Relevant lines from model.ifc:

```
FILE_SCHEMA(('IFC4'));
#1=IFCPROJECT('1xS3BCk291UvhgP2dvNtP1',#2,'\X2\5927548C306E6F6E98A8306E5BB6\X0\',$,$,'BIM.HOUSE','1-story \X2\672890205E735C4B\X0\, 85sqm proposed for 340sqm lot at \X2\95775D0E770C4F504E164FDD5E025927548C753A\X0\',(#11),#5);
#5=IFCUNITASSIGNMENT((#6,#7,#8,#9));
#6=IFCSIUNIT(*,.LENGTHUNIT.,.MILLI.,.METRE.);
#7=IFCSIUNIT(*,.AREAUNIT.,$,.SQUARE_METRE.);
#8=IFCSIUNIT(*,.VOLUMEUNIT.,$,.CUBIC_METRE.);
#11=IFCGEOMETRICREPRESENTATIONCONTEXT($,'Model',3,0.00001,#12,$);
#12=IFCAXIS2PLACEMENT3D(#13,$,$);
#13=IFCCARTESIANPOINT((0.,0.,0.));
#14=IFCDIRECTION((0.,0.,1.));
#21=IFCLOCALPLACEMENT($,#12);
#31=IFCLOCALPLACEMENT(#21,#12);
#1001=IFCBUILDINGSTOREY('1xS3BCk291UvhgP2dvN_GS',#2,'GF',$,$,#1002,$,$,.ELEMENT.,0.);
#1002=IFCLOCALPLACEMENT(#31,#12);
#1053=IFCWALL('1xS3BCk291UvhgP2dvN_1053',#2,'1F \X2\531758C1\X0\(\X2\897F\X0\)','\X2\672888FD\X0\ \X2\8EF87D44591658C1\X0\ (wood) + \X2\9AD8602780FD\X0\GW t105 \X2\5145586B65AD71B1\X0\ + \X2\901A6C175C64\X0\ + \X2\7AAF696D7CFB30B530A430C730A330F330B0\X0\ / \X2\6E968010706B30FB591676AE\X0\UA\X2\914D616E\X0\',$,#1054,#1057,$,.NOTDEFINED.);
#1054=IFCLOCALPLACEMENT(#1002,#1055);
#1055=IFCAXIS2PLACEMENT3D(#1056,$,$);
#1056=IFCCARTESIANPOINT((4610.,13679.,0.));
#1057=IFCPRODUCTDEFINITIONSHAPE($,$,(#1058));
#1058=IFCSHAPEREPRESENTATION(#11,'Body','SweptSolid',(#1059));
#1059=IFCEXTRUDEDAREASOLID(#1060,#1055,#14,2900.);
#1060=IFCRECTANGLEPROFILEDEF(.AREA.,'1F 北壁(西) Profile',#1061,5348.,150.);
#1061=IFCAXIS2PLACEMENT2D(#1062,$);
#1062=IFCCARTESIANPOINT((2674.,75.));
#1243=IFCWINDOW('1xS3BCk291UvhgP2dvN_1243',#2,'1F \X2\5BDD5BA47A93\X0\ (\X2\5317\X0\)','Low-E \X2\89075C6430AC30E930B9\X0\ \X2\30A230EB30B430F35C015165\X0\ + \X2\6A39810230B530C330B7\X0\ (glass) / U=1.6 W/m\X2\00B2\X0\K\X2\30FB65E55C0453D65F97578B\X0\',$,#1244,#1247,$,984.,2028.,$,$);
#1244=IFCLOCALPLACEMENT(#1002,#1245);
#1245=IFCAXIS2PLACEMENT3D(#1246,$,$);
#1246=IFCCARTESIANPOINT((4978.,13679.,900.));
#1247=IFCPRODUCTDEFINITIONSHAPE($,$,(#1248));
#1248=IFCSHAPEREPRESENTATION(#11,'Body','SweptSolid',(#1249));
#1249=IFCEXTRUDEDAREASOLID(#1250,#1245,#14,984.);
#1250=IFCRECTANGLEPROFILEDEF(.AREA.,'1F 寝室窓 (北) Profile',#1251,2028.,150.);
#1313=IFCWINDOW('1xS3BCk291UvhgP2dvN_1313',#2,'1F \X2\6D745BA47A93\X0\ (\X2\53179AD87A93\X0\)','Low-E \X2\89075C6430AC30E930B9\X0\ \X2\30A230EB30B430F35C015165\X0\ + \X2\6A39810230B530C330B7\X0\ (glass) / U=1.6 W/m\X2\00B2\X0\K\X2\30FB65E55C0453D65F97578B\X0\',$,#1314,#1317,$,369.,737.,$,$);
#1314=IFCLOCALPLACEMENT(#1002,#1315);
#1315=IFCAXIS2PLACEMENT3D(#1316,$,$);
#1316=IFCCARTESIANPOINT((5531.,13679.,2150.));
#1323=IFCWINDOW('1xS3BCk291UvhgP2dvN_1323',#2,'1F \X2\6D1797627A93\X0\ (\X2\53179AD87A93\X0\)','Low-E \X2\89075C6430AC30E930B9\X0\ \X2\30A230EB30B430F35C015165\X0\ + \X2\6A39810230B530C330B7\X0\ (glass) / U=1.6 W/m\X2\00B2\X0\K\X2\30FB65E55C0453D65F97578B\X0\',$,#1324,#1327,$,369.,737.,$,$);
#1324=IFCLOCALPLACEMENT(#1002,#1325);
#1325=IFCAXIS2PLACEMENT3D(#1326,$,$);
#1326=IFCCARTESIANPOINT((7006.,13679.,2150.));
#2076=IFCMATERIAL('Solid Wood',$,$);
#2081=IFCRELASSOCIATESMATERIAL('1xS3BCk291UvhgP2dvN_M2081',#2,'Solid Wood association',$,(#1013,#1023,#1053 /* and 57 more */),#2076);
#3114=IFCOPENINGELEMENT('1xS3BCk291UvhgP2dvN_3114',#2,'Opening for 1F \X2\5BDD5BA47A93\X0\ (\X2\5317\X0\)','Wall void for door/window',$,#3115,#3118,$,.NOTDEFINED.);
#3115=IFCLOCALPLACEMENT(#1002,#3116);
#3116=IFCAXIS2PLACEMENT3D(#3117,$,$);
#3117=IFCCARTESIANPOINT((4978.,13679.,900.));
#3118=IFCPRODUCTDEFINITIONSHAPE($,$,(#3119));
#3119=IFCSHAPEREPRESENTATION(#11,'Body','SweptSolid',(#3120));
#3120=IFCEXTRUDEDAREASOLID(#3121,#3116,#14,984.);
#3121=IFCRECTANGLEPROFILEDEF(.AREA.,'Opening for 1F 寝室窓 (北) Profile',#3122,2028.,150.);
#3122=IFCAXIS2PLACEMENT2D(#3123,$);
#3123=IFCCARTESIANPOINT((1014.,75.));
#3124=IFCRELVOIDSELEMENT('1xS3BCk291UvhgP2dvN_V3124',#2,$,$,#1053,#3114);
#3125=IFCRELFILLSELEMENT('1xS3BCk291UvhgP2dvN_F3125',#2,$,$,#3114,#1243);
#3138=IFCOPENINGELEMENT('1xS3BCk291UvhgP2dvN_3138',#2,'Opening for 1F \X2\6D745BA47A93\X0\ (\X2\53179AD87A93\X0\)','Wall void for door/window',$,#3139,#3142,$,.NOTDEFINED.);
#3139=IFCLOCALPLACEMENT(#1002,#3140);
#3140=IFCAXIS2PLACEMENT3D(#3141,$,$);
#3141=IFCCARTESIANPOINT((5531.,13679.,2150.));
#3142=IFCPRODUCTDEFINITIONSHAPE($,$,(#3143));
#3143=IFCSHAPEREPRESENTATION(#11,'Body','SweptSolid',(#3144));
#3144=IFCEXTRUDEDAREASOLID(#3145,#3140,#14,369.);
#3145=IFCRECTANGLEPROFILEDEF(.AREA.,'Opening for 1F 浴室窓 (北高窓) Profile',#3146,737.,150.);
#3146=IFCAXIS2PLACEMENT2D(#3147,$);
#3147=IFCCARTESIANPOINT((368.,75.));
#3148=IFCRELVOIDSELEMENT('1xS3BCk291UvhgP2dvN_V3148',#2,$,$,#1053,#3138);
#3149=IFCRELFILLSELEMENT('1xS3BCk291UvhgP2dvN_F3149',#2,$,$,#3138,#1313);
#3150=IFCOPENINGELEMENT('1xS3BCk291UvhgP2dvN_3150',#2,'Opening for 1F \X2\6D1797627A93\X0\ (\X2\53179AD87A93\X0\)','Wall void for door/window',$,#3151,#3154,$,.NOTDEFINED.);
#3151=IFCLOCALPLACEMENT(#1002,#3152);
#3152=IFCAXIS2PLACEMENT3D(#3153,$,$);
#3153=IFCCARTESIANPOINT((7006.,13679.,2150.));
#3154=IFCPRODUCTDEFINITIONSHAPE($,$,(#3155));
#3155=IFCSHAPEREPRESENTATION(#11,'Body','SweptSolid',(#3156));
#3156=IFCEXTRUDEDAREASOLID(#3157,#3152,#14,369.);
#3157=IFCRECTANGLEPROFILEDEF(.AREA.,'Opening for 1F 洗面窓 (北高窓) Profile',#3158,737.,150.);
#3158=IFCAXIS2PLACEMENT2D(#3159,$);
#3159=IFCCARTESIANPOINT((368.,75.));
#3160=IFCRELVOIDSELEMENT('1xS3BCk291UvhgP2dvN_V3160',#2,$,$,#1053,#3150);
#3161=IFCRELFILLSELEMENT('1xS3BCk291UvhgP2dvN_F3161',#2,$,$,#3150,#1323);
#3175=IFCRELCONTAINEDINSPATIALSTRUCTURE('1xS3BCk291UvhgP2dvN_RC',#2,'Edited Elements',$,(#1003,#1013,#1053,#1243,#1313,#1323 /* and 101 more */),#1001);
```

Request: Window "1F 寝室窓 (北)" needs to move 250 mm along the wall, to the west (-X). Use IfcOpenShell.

```python
import ifcopenshell
import ifcopenshell.api.geometry
import ifcopenshell.util.placement
import ifcopenshell.util.unit

model = ifcopenshell.open("model.ifc")
unit_scale = ifcopenshell.util.unit.calculate_unit_scale(model)

window = model.by_guid("1xS3BCk291UvhgP2dvN_1243")
opening = window.FillsVoids[0].RelatingOpeningElement
wall = opening.VoidsElements[0].RelatingBuildingElement

wall_matrix = ifcopenshell.util.placement.get_local_placement(wall.ObjectPlacement)
shift = wall_matrix[:3, 0] * -0.25 / unit_scale
before = ifcopenshell.util.placement.get_local_placement(window.ObjectPlacement)[:3, 3].copy()

# The window is not placed relative to its opening, so move both.
for product in (opening, window):
    matrix = ifcopenshell.util.placement.get_local_placement(product.ObjectPlacement)
    matrix[:3, 3] += shift
    ifcopenshell.api.geometry.edit_object_placement(model, product=product, matrix=matrix, is_si=False)

after = ifcopenshell.util.placement.get_local_placement(window.ObjectPlacement)[:3, 3]
print("window moved by", (after - before).round(3) + 0.0)

model.write("model_updated.ifc")
```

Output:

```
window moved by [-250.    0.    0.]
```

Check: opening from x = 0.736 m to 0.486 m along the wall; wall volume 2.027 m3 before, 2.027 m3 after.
